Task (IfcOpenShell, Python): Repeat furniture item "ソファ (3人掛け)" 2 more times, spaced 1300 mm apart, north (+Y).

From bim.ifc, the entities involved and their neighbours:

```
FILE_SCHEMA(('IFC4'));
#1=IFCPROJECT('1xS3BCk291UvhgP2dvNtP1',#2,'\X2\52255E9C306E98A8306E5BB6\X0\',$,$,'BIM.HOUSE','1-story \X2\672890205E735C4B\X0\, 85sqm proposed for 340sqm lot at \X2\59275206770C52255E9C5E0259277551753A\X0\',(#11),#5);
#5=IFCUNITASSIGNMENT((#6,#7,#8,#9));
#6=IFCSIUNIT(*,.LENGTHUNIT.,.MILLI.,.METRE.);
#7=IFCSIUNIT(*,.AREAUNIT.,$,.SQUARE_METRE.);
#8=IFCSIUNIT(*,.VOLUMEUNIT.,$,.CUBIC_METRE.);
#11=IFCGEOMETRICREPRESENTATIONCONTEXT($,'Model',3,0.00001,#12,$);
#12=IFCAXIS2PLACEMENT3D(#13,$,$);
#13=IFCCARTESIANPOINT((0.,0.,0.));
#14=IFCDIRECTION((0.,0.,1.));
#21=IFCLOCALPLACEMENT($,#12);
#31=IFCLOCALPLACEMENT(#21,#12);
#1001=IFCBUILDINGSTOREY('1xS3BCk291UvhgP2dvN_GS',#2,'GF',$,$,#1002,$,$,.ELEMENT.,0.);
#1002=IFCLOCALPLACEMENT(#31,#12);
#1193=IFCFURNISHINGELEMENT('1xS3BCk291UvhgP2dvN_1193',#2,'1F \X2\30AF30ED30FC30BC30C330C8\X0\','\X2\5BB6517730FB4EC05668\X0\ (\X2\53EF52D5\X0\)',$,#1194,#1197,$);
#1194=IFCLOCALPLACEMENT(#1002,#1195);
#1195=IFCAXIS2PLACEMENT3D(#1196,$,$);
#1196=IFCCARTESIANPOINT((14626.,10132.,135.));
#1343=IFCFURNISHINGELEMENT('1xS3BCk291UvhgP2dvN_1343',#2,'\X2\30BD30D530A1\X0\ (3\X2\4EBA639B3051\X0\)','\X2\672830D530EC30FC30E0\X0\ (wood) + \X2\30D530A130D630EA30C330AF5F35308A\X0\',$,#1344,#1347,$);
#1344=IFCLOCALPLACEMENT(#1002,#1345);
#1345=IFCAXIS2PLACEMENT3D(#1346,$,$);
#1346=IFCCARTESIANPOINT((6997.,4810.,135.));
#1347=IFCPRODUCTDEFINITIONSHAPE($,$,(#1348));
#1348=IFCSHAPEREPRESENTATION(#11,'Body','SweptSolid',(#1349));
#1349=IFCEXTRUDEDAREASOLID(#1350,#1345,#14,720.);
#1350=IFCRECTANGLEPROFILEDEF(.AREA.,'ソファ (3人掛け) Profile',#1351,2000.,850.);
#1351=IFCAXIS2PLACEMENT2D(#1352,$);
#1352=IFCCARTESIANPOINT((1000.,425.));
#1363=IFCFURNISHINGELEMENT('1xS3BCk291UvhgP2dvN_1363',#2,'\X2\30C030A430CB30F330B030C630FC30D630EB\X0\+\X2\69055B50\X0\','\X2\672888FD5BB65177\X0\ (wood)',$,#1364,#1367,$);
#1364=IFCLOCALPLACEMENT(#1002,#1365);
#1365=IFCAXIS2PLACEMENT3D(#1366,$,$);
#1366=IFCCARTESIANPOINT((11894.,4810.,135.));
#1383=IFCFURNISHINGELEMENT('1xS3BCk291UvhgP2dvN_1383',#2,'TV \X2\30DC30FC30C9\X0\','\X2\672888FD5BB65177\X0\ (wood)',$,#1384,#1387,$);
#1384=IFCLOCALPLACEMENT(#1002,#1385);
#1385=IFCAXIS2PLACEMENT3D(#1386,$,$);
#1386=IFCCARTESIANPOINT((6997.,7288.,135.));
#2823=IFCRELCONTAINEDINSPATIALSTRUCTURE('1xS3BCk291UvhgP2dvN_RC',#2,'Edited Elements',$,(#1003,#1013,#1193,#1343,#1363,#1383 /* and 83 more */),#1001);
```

```python
import numpy as np
import ifcopenshell
import ifcopenshell.api.geometry
import ifcopenshell.api.root
import ifcopenshell.util.element
import ifcopenshell.util.placement

model = ifcopenshell.open("bim.ifc")


def reuse_history(source, copy):
    """copy_class also copies each property set's owner history, people and application; keep the originals."""
    for rel in copy.IsDefinedBy:
        if rel.is_a("IfcRelDefinesByProperties") and (history := rel.RelatingPropertyDefinition.OwnerHistory):
            rel.RelatingPropertyDefinition.OwnerHistory = source.OwnerHistory
            ifcopenshell.util.element.remove_deep2(model, history)


source = model.by_guid("1xS3BCk291UvhgP2dvN_1343")
base = ifcopenshell.util.placement.get_local_placement(source.ObjectPlacement)
step = np.array([0.0, 1.0, 0.0]) * 1300.0

for i in range(1, 3):
    copy = ifcopenshell.api.root.copy_class(model, product=source)
    copy.Representation = ifcopenshell.util.element.copy_deep(
        model, source.Representation, exclude=["IfcGeometricRepresentationContext", "IfcRepresentationMap"]
    )
    reuse_history(source, copy)
    matrix = base.copy()
    matrix[:3, 3] += i * step
    print("added at", matrix[:3, 3].round(3) + 0.0)
    ifcopenshell.api.geometry.edit_object_placement(model, product=copy, matrix=matrix, is_si=False)

model.write("bim_v2.ifc")
```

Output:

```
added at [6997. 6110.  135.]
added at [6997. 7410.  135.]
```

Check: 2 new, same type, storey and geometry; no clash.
